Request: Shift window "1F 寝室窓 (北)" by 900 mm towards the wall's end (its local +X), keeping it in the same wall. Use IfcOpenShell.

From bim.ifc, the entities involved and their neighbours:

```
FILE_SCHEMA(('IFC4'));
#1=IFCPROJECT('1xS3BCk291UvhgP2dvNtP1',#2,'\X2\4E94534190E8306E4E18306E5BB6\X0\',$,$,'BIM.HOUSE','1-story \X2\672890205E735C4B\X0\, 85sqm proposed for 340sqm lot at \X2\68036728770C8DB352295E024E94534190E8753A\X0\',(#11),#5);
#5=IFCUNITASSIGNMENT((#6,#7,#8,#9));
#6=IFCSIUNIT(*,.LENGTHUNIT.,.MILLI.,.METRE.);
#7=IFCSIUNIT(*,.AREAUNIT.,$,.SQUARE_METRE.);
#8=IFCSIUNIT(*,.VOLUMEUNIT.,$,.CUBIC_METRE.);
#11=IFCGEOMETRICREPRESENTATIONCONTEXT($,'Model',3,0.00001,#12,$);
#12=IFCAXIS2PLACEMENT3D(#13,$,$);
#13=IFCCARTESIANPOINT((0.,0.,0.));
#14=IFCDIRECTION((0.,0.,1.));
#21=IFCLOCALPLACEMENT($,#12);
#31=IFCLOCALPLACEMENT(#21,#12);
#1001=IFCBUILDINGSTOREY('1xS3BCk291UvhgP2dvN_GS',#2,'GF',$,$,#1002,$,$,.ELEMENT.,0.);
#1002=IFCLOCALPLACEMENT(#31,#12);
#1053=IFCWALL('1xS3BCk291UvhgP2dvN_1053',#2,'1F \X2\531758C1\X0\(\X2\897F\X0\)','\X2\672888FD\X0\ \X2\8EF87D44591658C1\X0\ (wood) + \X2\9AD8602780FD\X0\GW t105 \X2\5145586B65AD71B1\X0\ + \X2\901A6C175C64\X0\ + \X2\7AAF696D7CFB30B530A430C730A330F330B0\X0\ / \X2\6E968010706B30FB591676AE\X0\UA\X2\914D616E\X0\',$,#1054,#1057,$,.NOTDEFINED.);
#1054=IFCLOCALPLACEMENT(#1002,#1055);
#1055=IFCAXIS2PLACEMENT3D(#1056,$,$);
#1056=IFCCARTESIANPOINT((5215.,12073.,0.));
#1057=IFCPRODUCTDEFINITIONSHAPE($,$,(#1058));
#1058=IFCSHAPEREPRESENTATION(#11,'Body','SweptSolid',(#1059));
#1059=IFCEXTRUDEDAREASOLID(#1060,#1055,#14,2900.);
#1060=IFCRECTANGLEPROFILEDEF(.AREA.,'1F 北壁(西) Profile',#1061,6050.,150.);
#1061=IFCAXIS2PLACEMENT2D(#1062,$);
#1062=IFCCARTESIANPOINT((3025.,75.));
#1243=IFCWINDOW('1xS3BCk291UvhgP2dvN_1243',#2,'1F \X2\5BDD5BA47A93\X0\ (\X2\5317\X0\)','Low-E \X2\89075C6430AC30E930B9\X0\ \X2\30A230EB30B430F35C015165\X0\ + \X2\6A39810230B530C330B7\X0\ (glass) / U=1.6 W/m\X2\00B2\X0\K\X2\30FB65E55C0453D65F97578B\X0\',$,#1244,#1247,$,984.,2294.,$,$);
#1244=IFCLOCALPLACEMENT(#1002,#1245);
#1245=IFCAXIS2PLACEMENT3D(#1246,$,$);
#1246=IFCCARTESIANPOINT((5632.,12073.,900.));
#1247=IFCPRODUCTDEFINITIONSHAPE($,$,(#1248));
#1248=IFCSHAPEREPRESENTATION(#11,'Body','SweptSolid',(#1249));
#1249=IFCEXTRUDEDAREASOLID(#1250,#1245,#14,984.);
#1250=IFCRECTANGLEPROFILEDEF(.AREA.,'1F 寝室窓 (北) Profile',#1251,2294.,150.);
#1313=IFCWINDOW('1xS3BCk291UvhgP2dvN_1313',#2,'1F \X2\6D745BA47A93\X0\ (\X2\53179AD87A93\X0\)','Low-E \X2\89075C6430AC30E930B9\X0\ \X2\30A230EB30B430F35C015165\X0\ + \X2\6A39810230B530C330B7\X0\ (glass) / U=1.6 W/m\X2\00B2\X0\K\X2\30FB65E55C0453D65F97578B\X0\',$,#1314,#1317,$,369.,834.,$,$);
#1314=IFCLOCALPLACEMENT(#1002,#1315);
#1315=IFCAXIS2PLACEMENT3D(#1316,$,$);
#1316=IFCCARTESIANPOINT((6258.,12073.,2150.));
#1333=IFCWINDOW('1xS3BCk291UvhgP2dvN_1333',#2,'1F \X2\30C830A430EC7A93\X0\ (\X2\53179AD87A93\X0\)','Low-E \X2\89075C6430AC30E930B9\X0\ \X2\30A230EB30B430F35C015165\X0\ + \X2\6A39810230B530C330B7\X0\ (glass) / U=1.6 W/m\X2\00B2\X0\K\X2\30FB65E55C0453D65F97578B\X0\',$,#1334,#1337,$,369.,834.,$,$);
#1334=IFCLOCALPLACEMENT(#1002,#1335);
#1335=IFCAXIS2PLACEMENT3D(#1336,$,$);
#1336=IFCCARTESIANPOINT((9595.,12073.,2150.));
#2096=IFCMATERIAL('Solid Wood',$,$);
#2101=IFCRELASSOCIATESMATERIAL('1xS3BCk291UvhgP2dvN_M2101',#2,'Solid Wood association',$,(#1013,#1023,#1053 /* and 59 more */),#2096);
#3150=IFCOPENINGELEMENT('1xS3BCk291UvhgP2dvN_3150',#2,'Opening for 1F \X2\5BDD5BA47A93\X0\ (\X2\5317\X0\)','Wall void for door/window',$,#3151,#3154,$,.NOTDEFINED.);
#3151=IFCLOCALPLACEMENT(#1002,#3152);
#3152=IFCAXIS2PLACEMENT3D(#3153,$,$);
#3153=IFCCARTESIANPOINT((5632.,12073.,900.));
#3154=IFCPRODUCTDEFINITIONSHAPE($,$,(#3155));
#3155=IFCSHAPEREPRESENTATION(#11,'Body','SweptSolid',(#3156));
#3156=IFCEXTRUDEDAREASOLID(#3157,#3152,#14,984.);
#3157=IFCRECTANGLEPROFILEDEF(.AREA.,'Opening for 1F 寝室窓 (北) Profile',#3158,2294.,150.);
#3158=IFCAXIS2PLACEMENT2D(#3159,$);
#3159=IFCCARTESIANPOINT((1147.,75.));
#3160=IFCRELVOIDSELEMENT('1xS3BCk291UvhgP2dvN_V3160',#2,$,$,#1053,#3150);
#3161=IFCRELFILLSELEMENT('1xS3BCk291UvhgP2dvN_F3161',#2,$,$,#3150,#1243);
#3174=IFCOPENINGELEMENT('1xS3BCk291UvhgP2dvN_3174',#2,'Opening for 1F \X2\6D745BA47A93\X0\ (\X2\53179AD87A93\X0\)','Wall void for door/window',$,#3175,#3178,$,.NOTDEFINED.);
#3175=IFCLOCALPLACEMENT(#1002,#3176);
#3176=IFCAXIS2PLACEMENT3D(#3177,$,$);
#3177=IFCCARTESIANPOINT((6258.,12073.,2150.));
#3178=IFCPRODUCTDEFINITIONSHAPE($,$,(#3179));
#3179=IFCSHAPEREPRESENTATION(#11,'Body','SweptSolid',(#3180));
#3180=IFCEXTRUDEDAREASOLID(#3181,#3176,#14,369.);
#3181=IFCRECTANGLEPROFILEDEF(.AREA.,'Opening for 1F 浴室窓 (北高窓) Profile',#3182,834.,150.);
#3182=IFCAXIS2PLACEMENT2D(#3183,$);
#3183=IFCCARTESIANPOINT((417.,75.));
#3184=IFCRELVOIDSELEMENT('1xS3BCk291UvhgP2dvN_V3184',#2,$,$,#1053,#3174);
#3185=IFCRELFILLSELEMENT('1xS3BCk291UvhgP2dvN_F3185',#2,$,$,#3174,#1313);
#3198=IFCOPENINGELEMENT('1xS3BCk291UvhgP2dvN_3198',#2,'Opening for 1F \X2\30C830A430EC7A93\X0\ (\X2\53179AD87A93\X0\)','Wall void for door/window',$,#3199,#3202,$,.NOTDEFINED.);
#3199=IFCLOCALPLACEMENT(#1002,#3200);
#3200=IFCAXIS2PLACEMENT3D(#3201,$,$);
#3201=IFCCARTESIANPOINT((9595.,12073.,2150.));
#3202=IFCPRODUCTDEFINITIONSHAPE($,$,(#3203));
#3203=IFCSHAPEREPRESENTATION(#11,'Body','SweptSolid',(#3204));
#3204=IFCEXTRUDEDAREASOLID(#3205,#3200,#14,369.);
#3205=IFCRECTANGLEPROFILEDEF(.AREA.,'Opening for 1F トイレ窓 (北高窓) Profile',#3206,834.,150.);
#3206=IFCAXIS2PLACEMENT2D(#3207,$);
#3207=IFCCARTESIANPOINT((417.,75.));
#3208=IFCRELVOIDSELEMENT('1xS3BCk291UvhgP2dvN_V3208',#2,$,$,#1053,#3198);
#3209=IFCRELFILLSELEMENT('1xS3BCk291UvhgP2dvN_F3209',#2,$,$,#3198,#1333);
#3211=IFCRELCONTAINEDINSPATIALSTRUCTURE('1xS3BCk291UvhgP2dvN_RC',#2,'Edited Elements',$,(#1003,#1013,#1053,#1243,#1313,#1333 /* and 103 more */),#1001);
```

```python
import ifcopenshell
import ifcopenshell.api.geometry
import ifcopenshell.util.placement
import ifcopenshell.util.unit

model = ifcopenshell.open("bim.ifc")
unit_scale = ifcopenshell.util.unit.calculate_unit_scale(model)

window = model.by_guid("1xS3BCk291UvhgP2dvN_1243")
opening = window.FillsVoids[0].RelatingOpeningElement
wall = opening.VoidsElements[0].RelatingBuildingElement

wall_matrix = ifcopenshell.util.placement.get_local_placement(wall.ObjectPlacement)
shift = wall_matrix[:3, 0] * 0.9 / unit_scale
before = ifcopenshell.util.placement.get_local_placement(window.ObjectPlacement)[:3, 3].copy()

# The window is not placed relative to its opening, so move both.
for product in (opening, window):
    matrix = ifcopenshell.util.placement.get_local_placement(product.ObjectPlacement)
    matrix[:3, 3] += shift
    ifcopenshell.api.geometry.edit_object_placement(model, product=product, matrix=matrix, is_si=False)

after = ifcopenshell.util.placement.get_local_placement(window.ObjectPlacement)[:3, 3]
print("window moved by", (after - before).round(3) + 0.0)

model.write("bim_rev.ifc")
```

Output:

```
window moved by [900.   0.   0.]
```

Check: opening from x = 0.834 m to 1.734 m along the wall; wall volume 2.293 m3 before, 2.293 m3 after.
